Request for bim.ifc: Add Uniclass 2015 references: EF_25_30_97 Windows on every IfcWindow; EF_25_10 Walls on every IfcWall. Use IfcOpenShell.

First a look at what the model holds.

```python
import ifcopenshell

model = ifcopenshell.open("bim.ifc")
print(model.schema)
print("classifications:", [c.Name for c in model.by_type("IfcClassification")])
for ifc_class in ("IfcDoor", "IfcRoof", "IfcStair", "IfcWall", "IfcWindow"):
    print(ifc_class, len(model.by_type(ifc_class)))
```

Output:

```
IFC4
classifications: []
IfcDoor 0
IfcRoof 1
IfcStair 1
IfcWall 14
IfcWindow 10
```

```python
import ifcopenshell
import ifcopenshell.api.classification

model = ifcopenshell.open("bim.ifc")

system = ifcopenshell.api.classification.add_classification(model, classification="Uniclass 2015")

codes = {
    "IfcWindow": ("EF_25_30_97", "Windows"),
    "IfcWall": ("EF_25_10", "Walls"),
}
for ifc_class, (code, name) in codes.items():
    products = model.by_type(ifc_class)
    ifcopenshell.api.classification.add_reference(
        model, products=products, classification=system, identification=code, name=name
    )
    print(code, len(products))

model.write("bim_edited.ifc")
```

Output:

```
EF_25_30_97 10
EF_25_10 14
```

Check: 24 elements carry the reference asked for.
